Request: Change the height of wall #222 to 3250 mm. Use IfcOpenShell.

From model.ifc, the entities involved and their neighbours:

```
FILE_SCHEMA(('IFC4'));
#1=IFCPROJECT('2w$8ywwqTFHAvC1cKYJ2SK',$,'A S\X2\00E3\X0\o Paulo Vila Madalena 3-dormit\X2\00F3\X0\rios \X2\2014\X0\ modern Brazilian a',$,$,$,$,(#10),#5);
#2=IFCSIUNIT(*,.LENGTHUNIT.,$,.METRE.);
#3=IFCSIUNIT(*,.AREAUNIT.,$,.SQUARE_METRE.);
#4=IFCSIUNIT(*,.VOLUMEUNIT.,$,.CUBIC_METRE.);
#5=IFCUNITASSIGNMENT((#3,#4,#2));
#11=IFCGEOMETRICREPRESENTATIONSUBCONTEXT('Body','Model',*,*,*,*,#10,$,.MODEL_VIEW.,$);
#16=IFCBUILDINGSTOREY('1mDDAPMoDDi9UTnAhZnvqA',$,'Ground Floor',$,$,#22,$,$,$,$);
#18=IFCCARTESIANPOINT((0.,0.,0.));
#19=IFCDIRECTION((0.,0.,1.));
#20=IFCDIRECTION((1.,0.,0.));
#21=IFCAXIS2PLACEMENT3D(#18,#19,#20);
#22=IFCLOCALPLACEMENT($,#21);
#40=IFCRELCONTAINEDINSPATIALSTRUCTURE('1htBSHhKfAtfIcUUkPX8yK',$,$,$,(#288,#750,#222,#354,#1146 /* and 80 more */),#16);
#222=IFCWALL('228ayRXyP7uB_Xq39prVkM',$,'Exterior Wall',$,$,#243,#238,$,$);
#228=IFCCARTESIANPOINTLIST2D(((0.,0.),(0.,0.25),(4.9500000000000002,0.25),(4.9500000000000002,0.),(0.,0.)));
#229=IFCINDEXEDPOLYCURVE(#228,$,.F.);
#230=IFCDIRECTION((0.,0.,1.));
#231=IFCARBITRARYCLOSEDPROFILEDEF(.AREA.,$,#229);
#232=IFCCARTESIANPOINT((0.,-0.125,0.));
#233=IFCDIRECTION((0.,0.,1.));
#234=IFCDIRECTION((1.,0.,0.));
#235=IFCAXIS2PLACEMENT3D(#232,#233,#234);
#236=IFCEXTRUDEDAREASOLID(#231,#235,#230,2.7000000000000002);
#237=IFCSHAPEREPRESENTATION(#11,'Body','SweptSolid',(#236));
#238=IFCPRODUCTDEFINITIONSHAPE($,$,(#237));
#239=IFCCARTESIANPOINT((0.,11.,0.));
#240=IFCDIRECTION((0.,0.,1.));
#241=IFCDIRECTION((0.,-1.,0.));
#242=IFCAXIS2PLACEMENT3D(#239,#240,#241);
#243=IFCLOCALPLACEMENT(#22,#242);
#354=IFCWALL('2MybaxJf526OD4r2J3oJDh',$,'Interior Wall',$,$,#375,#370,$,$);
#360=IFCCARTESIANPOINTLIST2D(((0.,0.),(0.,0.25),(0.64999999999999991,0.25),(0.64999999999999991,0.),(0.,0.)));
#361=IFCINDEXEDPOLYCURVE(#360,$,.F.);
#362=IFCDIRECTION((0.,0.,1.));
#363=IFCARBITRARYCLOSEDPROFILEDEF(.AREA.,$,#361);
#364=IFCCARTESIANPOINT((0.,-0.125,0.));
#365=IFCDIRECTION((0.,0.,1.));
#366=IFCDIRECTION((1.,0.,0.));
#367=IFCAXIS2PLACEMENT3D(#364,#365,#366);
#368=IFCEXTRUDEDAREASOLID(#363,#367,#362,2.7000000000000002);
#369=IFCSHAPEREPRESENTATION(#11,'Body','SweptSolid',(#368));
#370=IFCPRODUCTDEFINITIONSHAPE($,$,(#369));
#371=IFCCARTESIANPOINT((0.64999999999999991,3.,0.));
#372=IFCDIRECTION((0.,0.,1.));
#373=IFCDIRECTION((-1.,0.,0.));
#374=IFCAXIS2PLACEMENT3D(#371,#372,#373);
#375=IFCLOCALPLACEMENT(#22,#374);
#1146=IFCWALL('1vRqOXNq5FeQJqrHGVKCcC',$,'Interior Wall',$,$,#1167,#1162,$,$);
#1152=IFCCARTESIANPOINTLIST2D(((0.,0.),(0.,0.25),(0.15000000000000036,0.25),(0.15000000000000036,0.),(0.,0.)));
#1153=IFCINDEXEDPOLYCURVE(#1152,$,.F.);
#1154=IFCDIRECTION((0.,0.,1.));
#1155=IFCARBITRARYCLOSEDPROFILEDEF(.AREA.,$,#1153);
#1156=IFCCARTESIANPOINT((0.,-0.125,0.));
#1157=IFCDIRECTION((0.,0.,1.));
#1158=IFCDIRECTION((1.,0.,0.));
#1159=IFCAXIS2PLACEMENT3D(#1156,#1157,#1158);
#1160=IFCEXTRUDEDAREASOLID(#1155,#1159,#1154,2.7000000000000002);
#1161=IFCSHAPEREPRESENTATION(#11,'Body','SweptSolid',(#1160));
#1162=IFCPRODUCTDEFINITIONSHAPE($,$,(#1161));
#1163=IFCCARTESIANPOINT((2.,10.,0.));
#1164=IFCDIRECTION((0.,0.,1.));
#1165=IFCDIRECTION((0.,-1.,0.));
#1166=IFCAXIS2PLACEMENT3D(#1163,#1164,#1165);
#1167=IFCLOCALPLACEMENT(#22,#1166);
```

```python
import ifcopenshell
import ifcopenshell.geom
import ifcopenshell.util.representation
import ifcopenshell.util.shape

model = ifcopenshell.open("model.ifc")
settings = ifcopenshell.geom.settings()


def volume(element):
    """Net volume in cubic metres, openings subtracted."""
    shape = ifcopenshell.geom.create_shape(settings, element)
    return ifcopenshell.util.shape.get_volume(shape.geometry)


wall = model.by_guid("228ayRXyP7uB_Xq39prVkM")
before = volume(wall)

body = ifcopenshell.util.representation.get_representation(wall, "Model", "Body")
solid = body.Items[0]
old_height = solid.Depth
solid.Depth = 3.25
after = volume(wall)

print(f"height {old_height:g} -> {solid.Depth:g}, volume {before:.3f} -> {after:.3f} m3")

model.write("model_edited.ifc")
```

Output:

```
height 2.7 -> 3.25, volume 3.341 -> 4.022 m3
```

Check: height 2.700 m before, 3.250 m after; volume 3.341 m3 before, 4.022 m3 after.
